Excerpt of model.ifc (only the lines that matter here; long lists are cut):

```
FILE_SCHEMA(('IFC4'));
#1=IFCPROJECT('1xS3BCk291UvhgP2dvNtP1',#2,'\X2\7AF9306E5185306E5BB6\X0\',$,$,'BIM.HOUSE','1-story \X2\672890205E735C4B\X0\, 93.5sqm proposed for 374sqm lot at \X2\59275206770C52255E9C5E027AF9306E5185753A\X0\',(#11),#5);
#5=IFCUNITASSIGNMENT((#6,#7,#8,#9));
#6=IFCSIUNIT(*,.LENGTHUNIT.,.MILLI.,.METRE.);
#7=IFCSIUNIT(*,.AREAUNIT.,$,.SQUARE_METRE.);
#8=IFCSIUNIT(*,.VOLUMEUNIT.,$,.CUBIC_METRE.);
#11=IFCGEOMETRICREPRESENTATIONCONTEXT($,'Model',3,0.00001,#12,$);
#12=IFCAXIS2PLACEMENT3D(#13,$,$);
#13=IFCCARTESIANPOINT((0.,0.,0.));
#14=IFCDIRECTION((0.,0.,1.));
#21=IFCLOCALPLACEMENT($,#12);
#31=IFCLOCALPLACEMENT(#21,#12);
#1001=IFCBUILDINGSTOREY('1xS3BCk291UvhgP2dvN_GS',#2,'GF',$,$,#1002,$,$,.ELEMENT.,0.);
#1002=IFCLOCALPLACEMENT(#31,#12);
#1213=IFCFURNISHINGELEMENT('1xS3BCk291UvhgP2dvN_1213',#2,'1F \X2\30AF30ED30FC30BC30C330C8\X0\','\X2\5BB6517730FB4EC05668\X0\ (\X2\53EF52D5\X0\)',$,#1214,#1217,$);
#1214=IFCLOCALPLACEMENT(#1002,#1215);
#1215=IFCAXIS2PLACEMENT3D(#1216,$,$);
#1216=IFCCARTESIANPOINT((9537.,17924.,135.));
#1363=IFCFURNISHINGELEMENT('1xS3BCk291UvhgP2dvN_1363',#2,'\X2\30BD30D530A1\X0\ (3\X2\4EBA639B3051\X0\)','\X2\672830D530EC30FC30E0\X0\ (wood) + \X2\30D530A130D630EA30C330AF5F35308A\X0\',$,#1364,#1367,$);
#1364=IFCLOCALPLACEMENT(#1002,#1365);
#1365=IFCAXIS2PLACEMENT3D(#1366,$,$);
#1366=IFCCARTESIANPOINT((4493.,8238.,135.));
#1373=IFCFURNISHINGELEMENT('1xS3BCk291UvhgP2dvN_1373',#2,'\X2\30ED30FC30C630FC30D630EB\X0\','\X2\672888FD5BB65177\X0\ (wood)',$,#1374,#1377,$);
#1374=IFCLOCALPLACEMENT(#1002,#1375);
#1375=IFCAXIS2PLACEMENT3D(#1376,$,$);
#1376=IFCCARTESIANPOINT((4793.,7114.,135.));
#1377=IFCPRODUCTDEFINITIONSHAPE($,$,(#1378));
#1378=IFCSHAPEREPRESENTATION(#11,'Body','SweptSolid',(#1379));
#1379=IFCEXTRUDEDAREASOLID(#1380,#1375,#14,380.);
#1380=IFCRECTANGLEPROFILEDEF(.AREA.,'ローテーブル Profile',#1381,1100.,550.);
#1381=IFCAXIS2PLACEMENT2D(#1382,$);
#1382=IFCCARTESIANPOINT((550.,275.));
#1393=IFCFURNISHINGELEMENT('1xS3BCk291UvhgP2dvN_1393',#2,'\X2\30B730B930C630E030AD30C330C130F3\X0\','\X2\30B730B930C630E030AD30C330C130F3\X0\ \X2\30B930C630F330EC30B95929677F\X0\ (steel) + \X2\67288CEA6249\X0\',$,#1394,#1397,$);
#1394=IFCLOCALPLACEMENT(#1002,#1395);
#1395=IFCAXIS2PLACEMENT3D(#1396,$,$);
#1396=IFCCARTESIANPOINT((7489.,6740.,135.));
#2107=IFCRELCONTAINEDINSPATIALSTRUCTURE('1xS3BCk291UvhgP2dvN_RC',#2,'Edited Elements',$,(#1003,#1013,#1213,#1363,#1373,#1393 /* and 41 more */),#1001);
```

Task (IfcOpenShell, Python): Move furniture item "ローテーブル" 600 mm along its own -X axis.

```python
import ifcopenshell
import ifcopenshell.api.geometry
import ifcopenshell.util.placement

model = ifcopenshell.open("model.ifc")

item = model.by_id(1373)
matrix = ifcopenshell.util.placement.get_local_placement(item.ObjectPlacement)
matrix[:3, 3] -= matrix[:3, 0] * 600.0
ifcopenshell.api.geometry.edit_object_placement(model, product=item, matrix=matrix, is_si=False)

print(ifcopenshell.util.placement.get_local_placement(item.ObjectPlacement).round(3) + 0.0)

model.write("model_v2.ifc")
```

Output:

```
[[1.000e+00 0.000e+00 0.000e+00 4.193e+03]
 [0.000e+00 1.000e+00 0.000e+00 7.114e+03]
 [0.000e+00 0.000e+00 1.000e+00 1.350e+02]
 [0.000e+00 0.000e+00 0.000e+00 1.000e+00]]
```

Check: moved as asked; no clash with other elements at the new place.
